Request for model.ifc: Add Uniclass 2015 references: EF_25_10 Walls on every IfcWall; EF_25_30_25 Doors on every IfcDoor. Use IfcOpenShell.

First a look at what the model holds.

```python
import ifcopenshell

model = ifcopenshell.open("model.ifc")
print(model.schema)
print("classifications:", [c.Name for c in model.by_type("IfcClassification")])
for ifc_class in ("IfcDoor", "IfcRoof", "IfcStair", "IfcWall", "IfcWindow"):
    print(ifc_class, len(model.by_type(ifc_class)))
```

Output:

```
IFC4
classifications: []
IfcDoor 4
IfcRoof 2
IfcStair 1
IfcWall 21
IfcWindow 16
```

```python
import ifcopenshell
import ifcopenshell.api.classification

model = ifcopenshell.open("model.ifc")

system = ifcopenshell.api.classification.add_classification(model, classification="Uniclass 2015")

codes = {
    "IfcWall": ("EF_25_10", "Walls"),
    "IfcDoor": ("EF_25_30_25", "Doors"),
}
for ifc_class, (code, name) in codes.items():
    products = model.by_type(ifc_class)
    ifcopenshell.api.classification.add_reference(
        model, products=products, classification=system, identification=code, name=name
    )
    print(code, len(products))

model.write("model_updated.ifc")
```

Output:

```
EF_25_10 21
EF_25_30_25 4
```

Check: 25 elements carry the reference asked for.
